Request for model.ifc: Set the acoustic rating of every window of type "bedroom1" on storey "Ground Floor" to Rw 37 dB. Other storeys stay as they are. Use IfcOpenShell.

First a look at what the model holds.

```python
import ifcopenshell
import ifcopenshell.util.element

model = ifcopenshell.open("model.ifc")
print(model.schema)
storey = next(s for s in model.by_type("IfcBuildingStorey") if s.Name == "Ground Floor")
windows = [e for e in ifcopenshell.util.element.get_decomposition(storey) if e.is_a("IfcWindow")]
seen = {}
for e in windows:
    element_type = ifcopenshell.util.element.get_type(e)
    key = (element_type.Name if element_type != e and element_type else None, ifcopenshell.util.element.get_pset(e, "Pset_WindowCommon", "AcousticRating"))
    seen[key] = seen.get(key, 0) + 1
for (name, value), count in sorted(seen.items(), key=str):
    print(count, "x", name, "|", value)
```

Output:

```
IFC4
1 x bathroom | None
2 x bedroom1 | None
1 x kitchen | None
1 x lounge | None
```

```python
import ifcopenshell
import ifcopenshell.api.pset
import ifcopenshell.util.element

model = ifcopenshell.open("model.ifc")

storey = next(s for s in model.by_type("IfcBuildingStorey") if s.Name == "Ground Floor")
windows = [e for e in ifcopenshell.util.element.get_decomposition(storey) if e.is_a("IfcWindow")]

count = 0
for e in windows:
    element_type = ifcopenshell.util.element.get_type(e)
    if element_type in (None, e) or element_type.Name != "bedroom1":
        continue
    # add_pset returns the element's existing set when there is one.
    pset = ifcopenshell.api.pset.add_pset(model, product=e, name="Pset_WindowCommon")
    ifcopenshell.api.pset.edit_pset(model, pset=pset, properties={"AcousticRating": "Rw 37 dB"})
    count += 1

print(count, "windows updated")

model.write("model_updated.ifc")
```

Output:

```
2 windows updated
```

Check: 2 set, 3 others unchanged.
